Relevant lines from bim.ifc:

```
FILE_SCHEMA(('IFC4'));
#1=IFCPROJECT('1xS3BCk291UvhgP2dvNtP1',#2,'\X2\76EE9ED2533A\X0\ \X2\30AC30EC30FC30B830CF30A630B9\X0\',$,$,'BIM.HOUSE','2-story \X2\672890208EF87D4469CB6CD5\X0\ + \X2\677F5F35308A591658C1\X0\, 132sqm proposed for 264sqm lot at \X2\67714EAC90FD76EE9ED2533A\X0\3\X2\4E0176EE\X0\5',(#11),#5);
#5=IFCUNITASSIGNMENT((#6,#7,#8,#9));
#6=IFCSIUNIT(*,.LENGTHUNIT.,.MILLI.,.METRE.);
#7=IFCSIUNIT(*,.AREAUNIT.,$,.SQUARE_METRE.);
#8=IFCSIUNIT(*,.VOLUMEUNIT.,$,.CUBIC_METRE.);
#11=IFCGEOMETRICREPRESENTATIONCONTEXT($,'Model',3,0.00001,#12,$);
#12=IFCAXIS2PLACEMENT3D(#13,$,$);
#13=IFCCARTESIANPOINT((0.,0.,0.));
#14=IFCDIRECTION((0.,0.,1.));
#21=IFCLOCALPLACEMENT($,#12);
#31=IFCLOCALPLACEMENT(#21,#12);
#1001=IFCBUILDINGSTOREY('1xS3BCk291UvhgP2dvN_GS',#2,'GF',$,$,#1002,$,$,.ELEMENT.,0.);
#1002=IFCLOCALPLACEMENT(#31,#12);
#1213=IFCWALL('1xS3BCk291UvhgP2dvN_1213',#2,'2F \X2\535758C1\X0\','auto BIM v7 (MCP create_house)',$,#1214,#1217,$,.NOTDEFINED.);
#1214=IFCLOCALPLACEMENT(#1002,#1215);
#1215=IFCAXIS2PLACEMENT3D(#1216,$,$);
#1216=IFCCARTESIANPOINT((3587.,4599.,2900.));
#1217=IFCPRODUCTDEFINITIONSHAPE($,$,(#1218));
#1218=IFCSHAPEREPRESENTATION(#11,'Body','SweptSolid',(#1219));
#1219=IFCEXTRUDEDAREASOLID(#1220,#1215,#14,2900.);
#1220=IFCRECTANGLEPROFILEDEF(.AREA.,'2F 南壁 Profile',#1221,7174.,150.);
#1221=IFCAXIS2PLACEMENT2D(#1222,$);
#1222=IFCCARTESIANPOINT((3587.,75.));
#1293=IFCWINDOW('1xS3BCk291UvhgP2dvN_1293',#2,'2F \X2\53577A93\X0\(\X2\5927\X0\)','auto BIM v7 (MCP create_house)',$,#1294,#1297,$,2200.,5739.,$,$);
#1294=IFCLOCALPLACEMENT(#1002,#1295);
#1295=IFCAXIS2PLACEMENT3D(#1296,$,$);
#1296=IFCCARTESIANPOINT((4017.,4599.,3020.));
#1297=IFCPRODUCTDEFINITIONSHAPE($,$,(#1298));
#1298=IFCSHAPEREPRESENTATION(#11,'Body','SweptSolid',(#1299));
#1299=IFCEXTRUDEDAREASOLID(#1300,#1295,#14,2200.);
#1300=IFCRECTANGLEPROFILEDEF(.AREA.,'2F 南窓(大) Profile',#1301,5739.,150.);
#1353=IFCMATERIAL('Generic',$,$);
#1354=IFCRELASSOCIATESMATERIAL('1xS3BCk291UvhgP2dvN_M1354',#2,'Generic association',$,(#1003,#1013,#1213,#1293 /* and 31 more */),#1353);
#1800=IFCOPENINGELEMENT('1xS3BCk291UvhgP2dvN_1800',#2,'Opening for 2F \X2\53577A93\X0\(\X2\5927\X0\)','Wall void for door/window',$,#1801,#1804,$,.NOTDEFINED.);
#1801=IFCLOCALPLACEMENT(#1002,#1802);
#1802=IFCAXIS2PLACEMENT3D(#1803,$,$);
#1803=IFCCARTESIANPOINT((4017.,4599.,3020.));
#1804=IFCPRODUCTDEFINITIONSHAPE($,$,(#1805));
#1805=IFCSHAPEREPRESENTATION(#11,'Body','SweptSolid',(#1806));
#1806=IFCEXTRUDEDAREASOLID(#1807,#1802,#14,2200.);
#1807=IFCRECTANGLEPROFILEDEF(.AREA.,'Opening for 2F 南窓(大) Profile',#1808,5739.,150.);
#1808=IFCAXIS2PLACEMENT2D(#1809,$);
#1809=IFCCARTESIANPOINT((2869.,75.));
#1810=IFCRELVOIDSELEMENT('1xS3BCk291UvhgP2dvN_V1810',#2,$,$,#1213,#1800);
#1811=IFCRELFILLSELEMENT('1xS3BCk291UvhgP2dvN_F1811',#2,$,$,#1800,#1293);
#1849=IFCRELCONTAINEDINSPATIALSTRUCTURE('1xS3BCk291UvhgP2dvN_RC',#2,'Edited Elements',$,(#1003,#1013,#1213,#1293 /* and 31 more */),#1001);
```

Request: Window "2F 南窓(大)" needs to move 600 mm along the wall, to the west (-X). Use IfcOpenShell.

```python
import ifcopenshell
import ifcopenshell.api.geometry
import ifcopenshell.util.placement
import ifcopenshell.util.unit

model = ifcopenshell.open("bim.ifc")
unit_scale = ifcopenshell.util.unit.calculate_unit_scale(model)

window = model.by_id(1293)
opening = window.FillsVoids[0].RelatingOpeningElement
wall = opening.VoidsElements[0].RelatingBuildingElement

wall_matrix = ifcopenshell.util.placement.get_local_placement(wall.ObjectPlacement)
shift = wall_matrix[:3, 0] * -0.6 / unit_scale
before = ifcopenshell.util.placement.get_local_placement(window.ObjectPlacement)[:3, 3].copy()

# The window is not placed relative to its opening, so move both.
for product in (opening, window):
    matrix = ifcopenshell.util.placement.get_local_placement(product.ObjectPlacement)
    matrix[:3, 3] += shift
    ifcopenshell.api.geometry.edit_object_placement(model, product=product, matrix=matrix, is_si=False)

after = ifcopenshell.util.placement.get_local_placement(window.ObjectPlacement)[:3, 3]
print("window moved by", (after - before).round(3) + 0.0)

model.write("bim_rev.ifc")
```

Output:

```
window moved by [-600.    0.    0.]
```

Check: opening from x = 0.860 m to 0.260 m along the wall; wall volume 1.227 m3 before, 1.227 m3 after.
